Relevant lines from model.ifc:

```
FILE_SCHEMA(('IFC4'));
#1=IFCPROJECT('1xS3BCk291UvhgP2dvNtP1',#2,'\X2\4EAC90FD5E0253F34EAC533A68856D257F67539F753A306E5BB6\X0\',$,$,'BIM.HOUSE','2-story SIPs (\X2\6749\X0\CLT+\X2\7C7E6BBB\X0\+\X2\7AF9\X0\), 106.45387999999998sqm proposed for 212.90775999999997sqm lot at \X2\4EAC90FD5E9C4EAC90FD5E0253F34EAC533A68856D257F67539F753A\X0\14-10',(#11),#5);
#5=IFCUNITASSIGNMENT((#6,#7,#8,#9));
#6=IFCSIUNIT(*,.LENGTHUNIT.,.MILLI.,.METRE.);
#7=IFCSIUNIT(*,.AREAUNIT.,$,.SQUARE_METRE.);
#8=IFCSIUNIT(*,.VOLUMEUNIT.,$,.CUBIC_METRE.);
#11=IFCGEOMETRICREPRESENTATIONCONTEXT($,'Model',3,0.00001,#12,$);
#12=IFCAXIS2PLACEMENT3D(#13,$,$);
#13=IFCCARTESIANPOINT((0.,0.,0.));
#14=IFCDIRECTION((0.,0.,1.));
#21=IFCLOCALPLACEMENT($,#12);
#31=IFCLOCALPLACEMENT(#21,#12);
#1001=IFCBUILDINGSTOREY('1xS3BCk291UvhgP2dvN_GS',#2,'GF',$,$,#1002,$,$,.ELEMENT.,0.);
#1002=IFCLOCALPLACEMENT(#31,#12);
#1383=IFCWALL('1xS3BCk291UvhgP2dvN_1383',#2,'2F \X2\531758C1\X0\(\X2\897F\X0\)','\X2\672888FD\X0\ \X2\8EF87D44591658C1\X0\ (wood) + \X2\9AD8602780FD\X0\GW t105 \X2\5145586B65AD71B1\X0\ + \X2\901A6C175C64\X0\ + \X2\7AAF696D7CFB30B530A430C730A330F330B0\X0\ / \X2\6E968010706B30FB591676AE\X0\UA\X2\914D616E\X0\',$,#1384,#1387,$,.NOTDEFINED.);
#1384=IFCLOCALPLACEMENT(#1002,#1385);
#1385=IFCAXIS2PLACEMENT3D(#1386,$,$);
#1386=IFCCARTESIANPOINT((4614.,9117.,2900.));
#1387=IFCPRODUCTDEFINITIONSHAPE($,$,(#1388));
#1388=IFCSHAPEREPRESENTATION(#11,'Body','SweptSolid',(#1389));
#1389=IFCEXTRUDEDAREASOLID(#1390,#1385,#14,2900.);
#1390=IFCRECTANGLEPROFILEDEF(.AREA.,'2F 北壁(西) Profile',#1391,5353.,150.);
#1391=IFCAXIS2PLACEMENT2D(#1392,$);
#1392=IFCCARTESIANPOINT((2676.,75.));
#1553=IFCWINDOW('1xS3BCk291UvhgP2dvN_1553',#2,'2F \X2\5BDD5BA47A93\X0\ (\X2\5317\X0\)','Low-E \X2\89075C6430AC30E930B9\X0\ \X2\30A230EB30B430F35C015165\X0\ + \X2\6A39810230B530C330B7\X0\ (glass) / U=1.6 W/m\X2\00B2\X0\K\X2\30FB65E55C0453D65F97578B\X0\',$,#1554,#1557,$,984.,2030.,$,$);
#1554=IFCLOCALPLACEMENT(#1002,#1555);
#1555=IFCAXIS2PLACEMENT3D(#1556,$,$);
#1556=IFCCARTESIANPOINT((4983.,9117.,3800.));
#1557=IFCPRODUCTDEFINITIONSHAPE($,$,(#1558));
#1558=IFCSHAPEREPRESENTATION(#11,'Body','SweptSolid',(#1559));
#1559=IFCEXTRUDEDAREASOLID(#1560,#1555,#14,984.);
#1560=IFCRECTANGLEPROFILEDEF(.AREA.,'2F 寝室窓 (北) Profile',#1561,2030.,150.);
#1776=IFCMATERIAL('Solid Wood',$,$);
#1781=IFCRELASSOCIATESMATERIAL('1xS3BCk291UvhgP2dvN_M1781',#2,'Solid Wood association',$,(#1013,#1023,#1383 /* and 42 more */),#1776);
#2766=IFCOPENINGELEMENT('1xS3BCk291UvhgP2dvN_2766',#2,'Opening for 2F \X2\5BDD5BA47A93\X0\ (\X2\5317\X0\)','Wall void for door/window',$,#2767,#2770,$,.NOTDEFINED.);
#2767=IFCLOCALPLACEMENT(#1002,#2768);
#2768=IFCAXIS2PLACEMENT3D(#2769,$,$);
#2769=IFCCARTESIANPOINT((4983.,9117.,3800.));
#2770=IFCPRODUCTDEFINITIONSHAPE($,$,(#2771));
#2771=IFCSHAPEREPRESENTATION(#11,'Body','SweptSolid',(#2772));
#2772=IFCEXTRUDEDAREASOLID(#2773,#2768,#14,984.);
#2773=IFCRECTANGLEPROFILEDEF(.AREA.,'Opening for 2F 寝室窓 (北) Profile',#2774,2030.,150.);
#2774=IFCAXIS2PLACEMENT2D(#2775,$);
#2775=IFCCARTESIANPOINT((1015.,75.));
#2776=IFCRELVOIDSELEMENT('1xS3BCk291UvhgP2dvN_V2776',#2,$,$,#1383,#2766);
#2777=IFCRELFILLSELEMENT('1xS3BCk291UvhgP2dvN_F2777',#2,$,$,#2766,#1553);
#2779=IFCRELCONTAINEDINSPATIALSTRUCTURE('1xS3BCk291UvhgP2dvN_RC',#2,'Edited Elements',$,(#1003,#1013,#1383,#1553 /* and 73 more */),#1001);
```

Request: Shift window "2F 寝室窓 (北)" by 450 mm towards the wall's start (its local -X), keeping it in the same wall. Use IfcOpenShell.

```python
import ifcopenshell
import ifcopenshell.api.geometry
import ifcopenshell.util.placement

model = ifcopenshell.open("model.ifc")

window = model.by_guid("1xS3BCk291UvhgP2dvN_1553")
opening = window.FillsVoids[0].RelatingOpeningElement
wall = opening.VoidsElements[0].RelatingBuildingElement

wall_matrix = ifcopenshell.util.placement.get_local_placement(wall.ObjectPlacement)
shift = wall_matrix[:3, 0] * -450.0
before = ifcopenshell.util.placement.get_local_placement(window.ObjectPlacement)[:3, 3].copy()

# The window is not placed relative to its opening, so move both.
for product in (opening, window):
    matrix = ifcopenshell.util.placement.get_local_placement(product.ObjectPlacement)
    matrix[:3, 3] += shift
    ifcopenshell.api.geometry.edit_object_placement(model, product=product, matrix=matrix, is_si=False)

after = ifcopenshell.util.placement.get_local_placement(window.ObjectPlacement)[:3, 3]
print("window moved by", (after - before).round(3) + 0.0)

model.write("model-out.ifc")
```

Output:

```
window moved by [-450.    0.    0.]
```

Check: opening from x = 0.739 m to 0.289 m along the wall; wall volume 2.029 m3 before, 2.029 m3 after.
